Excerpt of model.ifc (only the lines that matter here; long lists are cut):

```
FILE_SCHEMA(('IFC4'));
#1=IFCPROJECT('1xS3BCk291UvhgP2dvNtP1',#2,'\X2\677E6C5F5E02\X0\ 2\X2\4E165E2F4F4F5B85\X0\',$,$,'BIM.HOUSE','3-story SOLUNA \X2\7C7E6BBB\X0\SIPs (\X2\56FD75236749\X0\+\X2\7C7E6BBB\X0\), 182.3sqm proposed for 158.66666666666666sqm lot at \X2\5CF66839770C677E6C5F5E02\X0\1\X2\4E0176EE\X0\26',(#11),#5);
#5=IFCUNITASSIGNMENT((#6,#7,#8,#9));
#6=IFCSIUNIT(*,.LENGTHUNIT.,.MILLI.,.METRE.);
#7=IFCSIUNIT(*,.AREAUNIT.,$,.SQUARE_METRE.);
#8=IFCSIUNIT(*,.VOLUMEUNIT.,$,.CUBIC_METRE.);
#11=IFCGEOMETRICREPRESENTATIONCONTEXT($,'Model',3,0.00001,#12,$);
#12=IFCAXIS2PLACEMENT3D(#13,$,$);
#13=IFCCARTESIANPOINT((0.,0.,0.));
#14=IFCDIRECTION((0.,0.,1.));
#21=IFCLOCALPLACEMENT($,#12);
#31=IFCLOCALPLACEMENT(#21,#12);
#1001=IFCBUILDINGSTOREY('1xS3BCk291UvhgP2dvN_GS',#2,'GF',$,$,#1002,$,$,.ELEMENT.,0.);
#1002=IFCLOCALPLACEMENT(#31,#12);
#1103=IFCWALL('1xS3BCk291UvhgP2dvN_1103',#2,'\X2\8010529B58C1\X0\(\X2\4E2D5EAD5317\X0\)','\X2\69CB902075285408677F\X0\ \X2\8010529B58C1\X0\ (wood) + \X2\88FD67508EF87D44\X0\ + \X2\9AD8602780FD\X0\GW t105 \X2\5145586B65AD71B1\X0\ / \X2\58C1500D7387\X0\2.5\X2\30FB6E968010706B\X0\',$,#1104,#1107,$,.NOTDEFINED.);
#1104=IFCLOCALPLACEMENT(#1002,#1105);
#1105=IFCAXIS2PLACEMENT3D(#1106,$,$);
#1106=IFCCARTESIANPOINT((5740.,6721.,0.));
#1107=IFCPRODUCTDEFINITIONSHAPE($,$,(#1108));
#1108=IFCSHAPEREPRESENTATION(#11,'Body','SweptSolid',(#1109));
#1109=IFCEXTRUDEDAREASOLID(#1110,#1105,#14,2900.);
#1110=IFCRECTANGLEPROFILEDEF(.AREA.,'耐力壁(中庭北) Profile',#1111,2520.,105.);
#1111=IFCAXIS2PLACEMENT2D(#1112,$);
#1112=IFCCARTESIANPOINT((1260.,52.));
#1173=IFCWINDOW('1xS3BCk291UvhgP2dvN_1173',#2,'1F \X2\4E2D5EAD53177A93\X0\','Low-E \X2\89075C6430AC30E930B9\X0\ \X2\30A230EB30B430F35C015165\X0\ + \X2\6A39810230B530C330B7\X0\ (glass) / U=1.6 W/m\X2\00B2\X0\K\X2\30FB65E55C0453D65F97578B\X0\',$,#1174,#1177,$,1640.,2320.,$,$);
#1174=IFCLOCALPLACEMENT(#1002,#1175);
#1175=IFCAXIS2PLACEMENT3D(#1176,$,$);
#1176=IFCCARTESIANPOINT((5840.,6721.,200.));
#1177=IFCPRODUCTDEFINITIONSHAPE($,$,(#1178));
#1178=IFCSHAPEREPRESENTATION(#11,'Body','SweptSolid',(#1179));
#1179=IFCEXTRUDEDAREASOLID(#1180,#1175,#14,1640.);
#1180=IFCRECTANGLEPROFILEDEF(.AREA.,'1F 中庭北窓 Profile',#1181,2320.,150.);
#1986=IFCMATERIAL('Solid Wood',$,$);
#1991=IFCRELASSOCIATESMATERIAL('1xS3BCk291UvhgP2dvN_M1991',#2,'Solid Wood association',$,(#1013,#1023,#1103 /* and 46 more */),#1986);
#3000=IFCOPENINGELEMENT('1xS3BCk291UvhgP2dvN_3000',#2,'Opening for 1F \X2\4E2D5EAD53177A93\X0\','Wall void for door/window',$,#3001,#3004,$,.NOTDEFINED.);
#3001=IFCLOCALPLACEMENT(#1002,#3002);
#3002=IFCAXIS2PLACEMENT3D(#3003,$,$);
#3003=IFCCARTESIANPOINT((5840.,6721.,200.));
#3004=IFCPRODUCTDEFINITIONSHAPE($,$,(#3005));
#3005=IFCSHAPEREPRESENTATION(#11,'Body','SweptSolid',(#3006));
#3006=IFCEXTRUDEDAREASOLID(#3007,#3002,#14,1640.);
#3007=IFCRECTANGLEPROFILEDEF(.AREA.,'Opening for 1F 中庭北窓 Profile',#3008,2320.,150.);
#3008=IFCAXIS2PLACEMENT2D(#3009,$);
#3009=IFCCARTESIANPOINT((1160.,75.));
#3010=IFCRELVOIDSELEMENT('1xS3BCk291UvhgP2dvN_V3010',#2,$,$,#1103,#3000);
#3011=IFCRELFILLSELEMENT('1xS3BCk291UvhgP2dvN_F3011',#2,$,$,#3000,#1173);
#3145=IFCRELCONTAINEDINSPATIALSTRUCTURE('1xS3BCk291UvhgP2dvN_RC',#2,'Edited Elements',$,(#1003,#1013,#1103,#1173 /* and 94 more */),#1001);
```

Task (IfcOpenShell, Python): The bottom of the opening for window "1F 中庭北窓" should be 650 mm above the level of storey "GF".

```python
import numpy as np
import ifcopenshell
import ifcopenshell.api.geometry
import ifcopenshell.geom
import ifcopenshell.util.element
import ifcopenshell.util.placement
import ifcopenshell.util.shape
import ifcopenshell.util.unit

model = ifcopenshell.open("model.ifc")
unit_scale = ifcopenshell.util.unit.calculate_unit_scale(model)

window = model.by_guid("1xS3BCk291UvhgP2dvN_1173")
opening = window.FillsVoids[0].RelatingOpeningElement
storey = ifcopenshell.util.element.get_container(window, ifc_class="IfcBuildingStorey")
level = ifcopenshell.util.placement.get_local_placement(storey.ObjectPlacement)[2, 3]

# The opening's origin need not be at the sill, so measure its lowest point.
shape = ifcopenshell.geom.create_shape(ifcopenshell.geom.settings(), opening)
bottom = ifcopenshell.util.shape.get_shape_bottom_elevation(shape, shape.geometry) / unit_scale
dz = level + 0.65 / unit_scale - bottom

shift = np.array([0.0, 0.0, dz])
# The window is not placed relative to its opening, so move both.
for product in (opening, window):
    matrix = ifcopenshell.util.placement.get_local_placement(product.ObjectPlacement)
    matrix[:3, 3] += shift
    ifcopenshell.api.geometry.edit_object_placement(model, product=product, matrix=matrix, is_si=False)

print(f"moved by {dz * unit_scale:+.3f} m")

model.write("model_rev.ifc")
```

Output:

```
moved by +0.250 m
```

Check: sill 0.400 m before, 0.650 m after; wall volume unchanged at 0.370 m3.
